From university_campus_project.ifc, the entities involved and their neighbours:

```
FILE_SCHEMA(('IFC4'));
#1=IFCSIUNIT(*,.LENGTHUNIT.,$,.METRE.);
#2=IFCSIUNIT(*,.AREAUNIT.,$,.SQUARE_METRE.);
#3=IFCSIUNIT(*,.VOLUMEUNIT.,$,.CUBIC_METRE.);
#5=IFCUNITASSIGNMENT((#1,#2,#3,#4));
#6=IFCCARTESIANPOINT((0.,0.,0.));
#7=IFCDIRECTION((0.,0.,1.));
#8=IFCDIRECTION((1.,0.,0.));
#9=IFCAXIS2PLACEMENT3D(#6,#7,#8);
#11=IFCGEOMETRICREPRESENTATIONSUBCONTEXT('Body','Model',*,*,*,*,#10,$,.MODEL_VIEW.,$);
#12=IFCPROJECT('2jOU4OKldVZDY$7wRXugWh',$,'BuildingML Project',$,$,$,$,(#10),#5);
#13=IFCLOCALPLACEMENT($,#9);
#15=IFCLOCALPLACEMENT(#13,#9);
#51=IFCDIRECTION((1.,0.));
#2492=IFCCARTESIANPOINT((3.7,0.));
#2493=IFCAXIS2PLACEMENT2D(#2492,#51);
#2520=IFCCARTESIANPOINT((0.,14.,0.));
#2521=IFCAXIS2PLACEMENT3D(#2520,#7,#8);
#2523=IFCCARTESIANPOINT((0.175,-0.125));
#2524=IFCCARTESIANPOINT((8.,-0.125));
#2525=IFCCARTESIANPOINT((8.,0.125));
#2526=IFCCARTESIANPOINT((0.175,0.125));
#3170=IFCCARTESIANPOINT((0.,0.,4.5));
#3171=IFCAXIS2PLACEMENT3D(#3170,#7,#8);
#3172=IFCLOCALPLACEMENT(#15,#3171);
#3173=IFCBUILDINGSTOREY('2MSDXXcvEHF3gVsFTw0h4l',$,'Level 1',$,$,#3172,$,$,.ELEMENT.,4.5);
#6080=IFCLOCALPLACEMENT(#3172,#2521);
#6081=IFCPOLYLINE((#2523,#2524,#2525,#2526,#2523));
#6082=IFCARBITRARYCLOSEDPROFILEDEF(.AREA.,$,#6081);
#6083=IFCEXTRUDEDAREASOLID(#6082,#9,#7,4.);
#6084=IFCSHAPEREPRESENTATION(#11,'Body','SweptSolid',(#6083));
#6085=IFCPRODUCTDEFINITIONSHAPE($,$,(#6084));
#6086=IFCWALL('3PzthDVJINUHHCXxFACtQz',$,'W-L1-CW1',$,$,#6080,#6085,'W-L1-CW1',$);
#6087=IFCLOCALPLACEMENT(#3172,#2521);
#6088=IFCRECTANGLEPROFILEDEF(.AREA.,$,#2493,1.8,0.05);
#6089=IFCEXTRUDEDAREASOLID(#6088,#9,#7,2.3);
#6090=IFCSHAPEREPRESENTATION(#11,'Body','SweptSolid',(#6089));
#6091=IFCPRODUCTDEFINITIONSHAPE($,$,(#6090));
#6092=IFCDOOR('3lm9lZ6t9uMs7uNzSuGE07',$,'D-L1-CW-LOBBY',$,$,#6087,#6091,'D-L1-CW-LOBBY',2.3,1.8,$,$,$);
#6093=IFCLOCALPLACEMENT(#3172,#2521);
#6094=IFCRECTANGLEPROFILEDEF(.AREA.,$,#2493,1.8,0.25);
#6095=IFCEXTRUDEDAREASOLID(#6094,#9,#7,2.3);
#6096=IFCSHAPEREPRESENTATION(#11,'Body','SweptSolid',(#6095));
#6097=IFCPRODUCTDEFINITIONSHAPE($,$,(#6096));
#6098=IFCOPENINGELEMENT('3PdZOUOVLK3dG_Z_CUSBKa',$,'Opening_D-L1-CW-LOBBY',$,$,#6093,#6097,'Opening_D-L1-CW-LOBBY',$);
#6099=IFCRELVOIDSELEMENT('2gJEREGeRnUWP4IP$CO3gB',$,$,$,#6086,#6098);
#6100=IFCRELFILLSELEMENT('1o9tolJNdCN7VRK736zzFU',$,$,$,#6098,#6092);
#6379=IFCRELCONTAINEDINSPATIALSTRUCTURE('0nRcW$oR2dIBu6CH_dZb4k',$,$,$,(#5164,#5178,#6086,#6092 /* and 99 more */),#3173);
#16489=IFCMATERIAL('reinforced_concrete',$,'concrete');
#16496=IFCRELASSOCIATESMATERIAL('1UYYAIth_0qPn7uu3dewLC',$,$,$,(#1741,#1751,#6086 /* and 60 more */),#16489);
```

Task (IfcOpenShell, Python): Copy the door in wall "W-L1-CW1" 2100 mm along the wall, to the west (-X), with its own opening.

```python
import ifcopenshell
import ifcopenshell.api.feature
import ifcopenshell.api.geometry
import ifcopenshell.api.root
import ifcopenshell.geom
import ifcopenshell.util.element
import ifcopenshell.util.placement
import ifcopenshell.util.shape

model = ifcopenshell.open("university_campus_project.ifc")
settings = ifcopenshell.geom.settings()


def volume(element):
    """Net volume in cubic metres, openings subtracted."""
    shape = ifcopenshell.geom.create_shape(settings, element)
    return ifcopenshell.util.shape.get_volume(shape.geometry)


door = model.by_guid("3lm9lZ6t9uMs7uNzSuGE07")
opening = door.FillsVoids[0].RelatingOpeningElement
wall = opening.VoidsElements[0].RelatingBuildingElement
before = volume(wall)
shift = ifcopenshell.util.placement.get_local_placement(wall.ObjectPlacement)[:3, 0] * -2.1

# copy_class copies the void relationship, type, container and properties, but no geometry.
new_opening = ifcopenshell.api.root.copy_class(model, product=opening)
new_opening.Representation = ifcopenshell.util.element.copy_deep(
    model, opening.Representation, exclude=["IfcGeometricRepresentationContext", "IfcRepresentationMap"]
)
new_opening.Tag = None
new_door = ifcopenshell.api.root.copy_class(model, product=door)
new_door.Representation = ifcopenshell.util.element.copy_deep(
    model, door.Representation, exclude=["IfcGeometricRepresentationContext", "IfcRepresentationMap"]
)
new_door.Tag = None
ifcopenshell.api.feature.add_filling(model, opening=new_opening, element=new_door)

for old, new in ((opening, new_opening), (door, new_door)):
    matrix = ifcopenshell.util.placement.get_local_placement(old.ObjectPlacement)
    matrix[:3, 3] += shift
    ifcopenshell.api.geometry.edit_object_placement(model, product=new, matrix=matrix, is_si=False)

after = volume(wall)

print(f"wall volume {before:.3f} -> {after:.3f} m3")

model.write("university_campus_project_rev.ifc")
```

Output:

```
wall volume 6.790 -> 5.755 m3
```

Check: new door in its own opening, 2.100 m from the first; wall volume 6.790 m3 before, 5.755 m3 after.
